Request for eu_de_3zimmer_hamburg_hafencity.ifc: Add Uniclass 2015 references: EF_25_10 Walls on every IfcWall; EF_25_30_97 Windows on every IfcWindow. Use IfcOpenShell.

First a look at what the model holds.

```python
import ifcopenshell

model = ifcopenshell.open("eu_de_3zimmer_hamburg_hafencity.ifc")
print(model.schema)
print("classifications:", [c.Name for c in model.by_type("IfcClassification")])
for ifc_class in ("IfcDoor", "IfcRoof", "IfcStair", "IfcWall", "IfcWindow"):
    print(ifc_class, len(model.by_type(ifc_class)))
```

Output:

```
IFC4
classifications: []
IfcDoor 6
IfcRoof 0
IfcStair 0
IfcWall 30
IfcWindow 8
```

```python
import ifcopenshell
import ifcopenshell.api.classification

model = ifcopenshell.open("eu_de_3zimmer_hamburg_hafencity.ifc")

system = ifcopenshell.api.classification.add_classification(model, classification="Uniclass 2015")

codes = {
    "IfcWall": ("EF_25_10", "Walls"),
    "IfcWindow": ("EF_25_30_97", "Windows"),
}
for ifc_class, (code, name) in codes.items():
    products = model.by_type(ifc_class)
    ifcopenshell.api.classification.add_reference(
        model, products=products, classification=system, identification=code, name=name
    )
    print(code, len(products))

model.write("eu_de_3zimmer_hamburg_hafencity_v2.ifc")
```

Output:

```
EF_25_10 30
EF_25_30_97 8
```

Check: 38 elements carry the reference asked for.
